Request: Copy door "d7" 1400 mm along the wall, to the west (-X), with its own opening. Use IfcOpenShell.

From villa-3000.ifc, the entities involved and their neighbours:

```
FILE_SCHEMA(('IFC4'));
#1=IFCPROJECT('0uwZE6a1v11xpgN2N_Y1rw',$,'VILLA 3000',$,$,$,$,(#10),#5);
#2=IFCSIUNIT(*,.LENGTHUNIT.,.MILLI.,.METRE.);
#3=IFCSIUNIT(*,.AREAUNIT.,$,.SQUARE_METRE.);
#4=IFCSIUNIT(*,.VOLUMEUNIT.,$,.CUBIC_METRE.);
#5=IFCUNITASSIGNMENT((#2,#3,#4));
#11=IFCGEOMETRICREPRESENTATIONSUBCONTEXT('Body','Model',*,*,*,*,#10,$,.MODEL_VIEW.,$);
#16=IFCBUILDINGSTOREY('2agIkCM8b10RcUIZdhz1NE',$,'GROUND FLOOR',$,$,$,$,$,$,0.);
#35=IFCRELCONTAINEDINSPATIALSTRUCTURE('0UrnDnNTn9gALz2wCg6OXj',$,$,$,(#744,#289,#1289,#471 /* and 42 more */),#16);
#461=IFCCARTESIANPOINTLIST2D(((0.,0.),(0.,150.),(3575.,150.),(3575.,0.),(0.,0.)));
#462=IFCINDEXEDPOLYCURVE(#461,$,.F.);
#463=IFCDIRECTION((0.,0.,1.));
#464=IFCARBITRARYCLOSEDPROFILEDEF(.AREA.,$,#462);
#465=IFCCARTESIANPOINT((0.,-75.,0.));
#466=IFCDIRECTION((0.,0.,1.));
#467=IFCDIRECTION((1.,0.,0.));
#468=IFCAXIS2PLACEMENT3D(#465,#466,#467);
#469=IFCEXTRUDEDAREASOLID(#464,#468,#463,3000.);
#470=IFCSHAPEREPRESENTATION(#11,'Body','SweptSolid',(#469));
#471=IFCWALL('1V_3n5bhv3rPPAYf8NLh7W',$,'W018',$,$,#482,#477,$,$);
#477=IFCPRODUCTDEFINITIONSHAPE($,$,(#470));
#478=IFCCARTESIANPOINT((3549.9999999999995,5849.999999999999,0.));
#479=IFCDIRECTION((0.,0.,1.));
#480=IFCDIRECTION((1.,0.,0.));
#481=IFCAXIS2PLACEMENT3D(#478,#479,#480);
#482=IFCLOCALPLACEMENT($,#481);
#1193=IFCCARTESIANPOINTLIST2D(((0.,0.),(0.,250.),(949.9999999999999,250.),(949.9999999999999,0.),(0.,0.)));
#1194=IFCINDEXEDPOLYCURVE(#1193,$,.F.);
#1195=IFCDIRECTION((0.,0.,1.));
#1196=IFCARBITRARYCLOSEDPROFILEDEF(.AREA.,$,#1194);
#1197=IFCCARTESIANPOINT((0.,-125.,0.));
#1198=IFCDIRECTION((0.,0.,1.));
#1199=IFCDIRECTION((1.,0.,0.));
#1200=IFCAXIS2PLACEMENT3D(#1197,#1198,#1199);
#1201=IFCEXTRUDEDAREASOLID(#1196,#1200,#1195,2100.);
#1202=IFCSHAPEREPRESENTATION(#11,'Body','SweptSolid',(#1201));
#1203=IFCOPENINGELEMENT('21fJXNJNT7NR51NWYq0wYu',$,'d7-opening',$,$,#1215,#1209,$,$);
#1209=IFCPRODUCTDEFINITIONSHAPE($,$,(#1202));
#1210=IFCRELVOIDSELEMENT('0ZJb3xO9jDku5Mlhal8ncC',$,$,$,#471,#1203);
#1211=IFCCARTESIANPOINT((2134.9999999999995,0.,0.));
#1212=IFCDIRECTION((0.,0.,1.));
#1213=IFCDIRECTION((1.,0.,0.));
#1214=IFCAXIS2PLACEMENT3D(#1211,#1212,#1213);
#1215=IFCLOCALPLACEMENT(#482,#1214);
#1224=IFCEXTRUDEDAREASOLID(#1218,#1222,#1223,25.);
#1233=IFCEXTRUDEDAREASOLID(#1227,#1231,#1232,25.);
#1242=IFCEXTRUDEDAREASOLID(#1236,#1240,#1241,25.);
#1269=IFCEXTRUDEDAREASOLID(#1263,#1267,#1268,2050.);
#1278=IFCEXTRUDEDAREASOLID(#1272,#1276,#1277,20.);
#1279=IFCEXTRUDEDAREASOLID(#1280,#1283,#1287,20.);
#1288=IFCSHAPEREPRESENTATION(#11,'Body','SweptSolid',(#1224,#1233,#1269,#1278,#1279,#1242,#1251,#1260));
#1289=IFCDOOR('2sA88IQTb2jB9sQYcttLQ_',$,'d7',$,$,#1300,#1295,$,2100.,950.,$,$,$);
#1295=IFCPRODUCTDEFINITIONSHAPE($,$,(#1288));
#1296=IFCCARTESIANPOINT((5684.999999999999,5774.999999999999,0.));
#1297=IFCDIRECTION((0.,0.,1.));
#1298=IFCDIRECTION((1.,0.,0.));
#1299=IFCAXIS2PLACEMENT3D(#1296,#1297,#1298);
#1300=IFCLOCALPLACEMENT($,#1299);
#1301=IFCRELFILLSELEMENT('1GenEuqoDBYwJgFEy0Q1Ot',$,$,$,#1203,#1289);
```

```python
import ifcopenshell
import ifcopenshell.api.feature
import ifcopenshell.api.geometry
import ifcopenshell.api.root
import ifcopenshell.geom
import ifcopenshell.util.element
import ifcopenshell.util.placement
import ifcopenshell.util.shape
import ifcopenshell.util.unit

model = ifcopenshell.open("villa-3000.ifc")
unit_scale = ifcopenshell.util.unit.calculate_unit_scale(model)
settings = ifcopenshell.geom.settings()


def volume(element):
    """Net volume in cubic metres, openings subtracted."""
    shape = ifcopenshell.geom.create_shape(settings, element)
    return ifcopenshell.util.shape.get_volume(shape.geometry)


door = model.by_guid("2sA88IQTb2jB9sQYcttLQ_")
opening = door.FillsVoids[0].RelatingOpeningElement
wall = opening.VoidsElements[0].RelatingBuildingElement
before = volume(wall)
shift = ifcopenshell.util.placement.get_local_placement(wall.ObjectPlacement)[:3, 0] * -1.4 / unit_scale

# copy_class copies the void relationship, type, container and properties, but no geometry.
new_opening = ifcopenshell.api.root.copy_class(model, product=opening)
new_opening.Representation = ifcopenshell.util.element.copy_deep(
    model, opening.Representation, exclude=["IfcGeometricRepresentationContext", "IfcRepresentationMap"]
)
new_door = ifcopenshell.api.root.copy_class(model, product=door)
new_door.Representation = ifcopenshell.util.element.copy_deep(
    model, door.Representation, exclude=["IfcGeometricRepresentationContext", "IfcRepresentationMap"]
)
ifcopenshell.api.feature.add_filling(model, opening=new_opening, element=new_door)

for old, new in ((opening, new_opening), (door, new_door)):
    matrix = ifcopenshell.util.placement.get_local_placement(old.ObjectPlacement)
    matrix[:3, 3] += shift
    ifcopenshell.api.geometry.edit_object_placement(model, product=new, matrix=matrix, is_si=False)

after = volume(wall)

print(f"wall volume {before:.3f} -> {after:.3f} m3")

model.write("villa-3000-out.ifc")
```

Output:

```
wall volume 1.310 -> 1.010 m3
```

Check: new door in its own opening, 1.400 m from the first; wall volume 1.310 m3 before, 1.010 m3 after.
